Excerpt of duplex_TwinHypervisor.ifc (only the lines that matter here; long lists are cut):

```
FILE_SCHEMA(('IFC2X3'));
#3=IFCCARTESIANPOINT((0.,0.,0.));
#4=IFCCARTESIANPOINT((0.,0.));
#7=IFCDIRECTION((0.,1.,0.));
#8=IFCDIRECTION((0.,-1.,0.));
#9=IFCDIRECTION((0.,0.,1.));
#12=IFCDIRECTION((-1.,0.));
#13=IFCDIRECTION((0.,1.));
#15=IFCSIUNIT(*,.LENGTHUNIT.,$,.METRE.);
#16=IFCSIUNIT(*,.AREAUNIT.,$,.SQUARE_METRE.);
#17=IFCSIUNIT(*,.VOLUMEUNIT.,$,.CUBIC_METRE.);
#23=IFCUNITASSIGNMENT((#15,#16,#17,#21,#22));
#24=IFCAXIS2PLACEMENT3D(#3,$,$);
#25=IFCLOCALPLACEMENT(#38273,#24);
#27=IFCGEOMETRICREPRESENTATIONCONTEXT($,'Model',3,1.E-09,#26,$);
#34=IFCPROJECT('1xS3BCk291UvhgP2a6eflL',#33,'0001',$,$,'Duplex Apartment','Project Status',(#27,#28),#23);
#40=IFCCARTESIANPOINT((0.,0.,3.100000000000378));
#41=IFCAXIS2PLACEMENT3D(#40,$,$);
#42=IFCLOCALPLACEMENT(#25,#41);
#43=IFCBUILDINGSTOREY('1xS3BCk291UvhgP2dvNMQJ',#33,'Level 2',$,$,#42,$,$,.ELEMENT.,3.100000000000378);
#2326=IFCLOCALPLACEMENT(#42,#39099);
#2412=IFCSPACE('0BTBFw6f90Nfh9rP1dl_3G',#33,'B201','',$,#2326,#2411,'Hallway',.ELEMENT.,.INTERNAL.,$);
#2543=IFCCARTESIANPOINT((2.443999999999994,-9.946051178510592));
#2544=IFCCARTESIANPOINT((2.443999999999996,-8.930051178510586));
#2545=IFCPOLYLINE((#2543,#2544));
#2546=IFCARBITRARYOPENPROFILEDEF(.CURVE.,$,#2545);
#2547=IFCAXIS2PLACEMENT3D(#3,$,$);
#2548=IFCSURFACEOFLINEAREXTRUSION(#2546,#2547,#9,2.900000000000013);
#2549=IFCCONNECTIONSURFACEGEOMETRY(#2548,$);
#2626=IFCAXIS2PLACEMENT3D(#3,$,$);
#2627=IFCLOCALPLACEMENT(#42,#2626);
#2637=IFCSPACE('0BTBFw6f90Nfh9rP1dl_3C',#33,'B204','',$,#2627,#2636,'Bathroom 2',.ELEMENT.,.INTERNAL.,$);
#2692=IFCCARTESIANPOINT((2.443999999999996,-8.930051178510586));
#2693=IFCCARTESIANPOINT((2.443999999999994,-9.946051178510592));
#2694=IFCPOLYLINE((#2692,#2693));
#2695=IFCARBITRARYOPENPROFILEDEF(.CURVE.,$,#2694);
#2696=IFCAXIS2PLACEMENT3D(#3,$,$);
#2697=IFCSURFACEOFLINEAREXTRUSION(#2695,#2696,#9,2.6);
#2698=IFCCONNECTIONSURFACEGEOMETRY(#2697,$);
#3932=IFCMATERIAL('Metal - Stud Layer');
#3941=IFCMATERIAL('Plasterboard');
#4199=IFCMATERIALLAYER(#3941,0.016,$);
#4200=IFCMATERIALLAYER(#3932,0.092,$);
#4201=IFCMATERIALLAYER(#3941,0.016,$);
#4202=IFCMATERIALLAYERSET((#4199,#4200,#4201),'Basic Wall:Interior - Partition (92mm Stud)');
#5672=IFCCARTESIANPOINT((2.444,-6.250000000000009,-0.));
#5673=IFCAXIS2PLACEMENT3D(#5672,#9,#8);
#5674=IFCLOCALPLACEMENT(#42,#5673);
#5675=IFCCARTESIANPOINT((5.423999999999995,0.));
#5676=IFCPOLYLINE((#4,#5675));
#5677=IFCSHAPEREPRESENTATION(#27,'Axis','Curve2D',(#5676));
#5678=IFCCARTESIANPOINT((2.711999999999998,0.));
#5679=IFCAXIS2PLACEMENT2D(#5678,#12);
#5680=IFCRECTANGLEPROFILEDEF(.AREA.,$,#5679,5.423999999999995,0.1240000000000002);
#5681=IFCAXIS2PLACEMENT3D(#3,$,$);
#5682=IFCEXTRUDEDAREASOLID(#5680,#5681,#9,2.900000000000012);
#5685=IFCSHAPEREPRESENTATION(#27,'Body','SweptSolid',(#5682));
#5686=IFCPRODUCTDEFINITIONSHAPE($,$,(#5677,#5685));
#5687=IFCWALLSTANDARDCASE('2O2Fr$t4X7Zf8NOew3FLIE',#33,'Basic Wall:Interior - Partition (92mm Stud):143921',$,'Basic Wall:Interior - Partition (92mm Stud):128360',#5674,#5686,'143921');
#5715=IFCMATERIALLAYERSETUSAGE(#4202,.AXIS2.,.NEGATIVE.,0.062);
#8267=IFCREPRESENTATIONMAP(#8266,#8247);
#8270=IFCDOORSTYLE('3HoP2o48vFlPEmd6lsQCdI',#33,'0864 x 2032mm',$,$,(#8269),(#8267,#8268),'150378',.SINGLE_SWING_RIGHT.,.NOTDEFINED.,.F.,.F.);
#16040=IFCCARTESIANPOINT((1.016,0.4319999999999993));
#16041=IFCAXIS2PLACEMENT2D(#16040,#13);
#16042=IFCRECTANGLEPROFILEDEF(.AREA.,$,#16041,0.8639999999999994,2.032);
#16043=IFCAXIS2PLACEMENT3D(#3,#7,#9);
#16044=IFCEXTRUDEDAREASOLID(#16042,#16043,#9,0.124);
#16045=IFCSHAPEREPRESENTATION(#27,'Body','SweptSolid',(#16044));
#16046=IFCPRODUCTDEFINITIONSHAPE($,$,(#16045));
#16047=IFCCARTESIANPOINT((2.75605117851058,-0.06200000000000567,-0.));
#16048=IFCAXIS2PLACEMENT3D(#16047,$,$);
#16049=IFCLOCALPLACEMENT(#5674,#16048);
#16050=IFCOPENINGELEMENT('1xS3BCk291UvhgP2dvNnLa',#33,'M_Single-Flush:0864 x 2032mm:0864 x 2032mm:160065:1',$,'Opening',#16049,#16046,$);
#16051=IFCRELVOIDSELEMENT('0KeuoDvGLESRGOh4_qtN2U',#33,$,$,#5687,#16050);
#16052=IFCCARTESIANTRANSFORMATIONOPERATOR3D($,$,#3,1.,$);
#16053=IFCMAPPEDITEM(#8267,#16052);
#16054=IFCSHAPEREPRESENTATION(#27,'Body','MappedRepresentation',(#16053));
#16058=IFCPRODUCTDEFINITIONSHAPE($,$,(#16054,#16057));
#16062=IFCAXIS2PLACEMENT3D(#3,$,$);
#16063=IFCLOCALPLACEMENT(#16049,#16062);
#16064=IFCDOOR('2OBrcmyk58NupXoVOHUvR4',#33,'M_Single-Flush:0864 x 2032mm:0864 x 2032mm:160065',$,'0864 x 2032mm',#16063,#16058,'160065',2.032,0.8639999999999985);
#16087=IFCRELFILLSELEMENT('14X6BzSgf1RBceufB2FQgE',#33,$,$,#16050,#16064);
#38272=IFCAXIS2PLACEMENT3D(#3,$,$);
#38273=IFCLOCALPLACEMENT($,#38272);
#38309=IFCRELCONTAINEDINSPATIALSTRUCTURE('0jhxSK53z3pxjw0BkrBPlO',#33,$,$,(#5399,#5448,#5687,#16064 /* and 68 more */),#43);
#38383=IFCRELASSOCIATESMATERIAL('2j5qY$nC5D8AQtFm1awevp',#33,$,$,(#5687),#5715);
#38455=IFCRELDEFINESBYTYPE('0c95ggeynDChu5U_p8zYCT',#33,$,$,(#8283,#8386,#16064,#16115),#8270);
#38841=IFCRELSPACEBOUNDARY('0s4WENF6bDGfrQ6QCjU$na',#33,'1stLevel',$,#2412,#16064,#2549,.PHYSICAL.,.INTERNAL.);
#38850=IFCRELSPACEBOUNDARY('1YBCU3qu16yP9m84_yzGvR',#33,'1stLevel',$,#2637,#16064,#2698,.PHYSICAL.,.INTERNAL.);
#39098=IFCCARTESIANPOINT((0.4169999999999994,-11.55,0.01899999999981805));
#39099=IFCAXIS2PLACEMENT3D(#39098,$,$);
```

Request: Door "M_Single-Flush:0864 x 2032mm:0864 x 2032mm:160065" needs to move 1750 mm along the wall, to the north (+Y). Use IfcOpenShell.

```python
import numpy as np
import ifcopenshell
import ifcopenshell.api.geometry
import ifcopenshell.util.placement
import ifcopenshell.util.unit

model = ifcopenshell.open("duplex_TwinHypervisor.ifc")
unit_scale = ifcopenshell.util.unit.calculate_unit_scale(model)

door = model.by_id(16064)
opening = door.FillsVoids[0].RelatingOpeningElement
wall = opening.VoidsElements[0].RelatingBuildingElement

wall_matrix = ifcopenshell.util.placement.get_local_placement(wall.ObjectPlacement)
shift = wall_matrix[:3, 0] * -1.75 / unit_scale
before = ifcopenshell.util.placement.get_local_placement(door.ObjectPlacement)[:3, 3].copy()

# The door is placed relative to its opening, so it follows when the opening moves.
matrix = ifcopenshell.util.placement.get_local_placement(opening.ObjectPlacement)
matrix[:3, 3] += shift
ifcopenshell.api.geometry.edit_object_placement(
    model, product=opening, matrix=matrix, is_si=False, should_transform_children=True
)

# Space boundary surfaces are stored in each space's coordinates; move them too.
for rel in door.ProvidesBoundaries:
    if not rel.ConnectionGeometry:
        continue
    surface = rel.ConnectionGeometry.SurfaceOnRelatingElement
    space_matrix = ifcopenshell.util.placement.get_local_placement(rel.RelatingSpace.ObjectPlacement)
    point = np.array(surface.Position.Location.Coordinates) + space_matrix[:3, :3].T @ shift
    surface.Position = model.createIfcAxis2Placement3D(
        model.createIfcCartesianPoint(point.tolist()), surface.Position.Axis, surface.Position.RefDirection
    )

after = ifcopenshell.util.placement.get_local_placement(door.ObjectPlacement)[:3, 3]
print("door moved by", (after - before).round(3) + 0.0)

model.write("duplex_TwinHypervisor_v2.ifc")
```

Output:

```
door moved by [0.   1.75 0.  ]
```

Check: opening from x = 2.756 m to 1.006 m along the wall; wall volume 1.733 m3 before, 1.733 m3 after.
